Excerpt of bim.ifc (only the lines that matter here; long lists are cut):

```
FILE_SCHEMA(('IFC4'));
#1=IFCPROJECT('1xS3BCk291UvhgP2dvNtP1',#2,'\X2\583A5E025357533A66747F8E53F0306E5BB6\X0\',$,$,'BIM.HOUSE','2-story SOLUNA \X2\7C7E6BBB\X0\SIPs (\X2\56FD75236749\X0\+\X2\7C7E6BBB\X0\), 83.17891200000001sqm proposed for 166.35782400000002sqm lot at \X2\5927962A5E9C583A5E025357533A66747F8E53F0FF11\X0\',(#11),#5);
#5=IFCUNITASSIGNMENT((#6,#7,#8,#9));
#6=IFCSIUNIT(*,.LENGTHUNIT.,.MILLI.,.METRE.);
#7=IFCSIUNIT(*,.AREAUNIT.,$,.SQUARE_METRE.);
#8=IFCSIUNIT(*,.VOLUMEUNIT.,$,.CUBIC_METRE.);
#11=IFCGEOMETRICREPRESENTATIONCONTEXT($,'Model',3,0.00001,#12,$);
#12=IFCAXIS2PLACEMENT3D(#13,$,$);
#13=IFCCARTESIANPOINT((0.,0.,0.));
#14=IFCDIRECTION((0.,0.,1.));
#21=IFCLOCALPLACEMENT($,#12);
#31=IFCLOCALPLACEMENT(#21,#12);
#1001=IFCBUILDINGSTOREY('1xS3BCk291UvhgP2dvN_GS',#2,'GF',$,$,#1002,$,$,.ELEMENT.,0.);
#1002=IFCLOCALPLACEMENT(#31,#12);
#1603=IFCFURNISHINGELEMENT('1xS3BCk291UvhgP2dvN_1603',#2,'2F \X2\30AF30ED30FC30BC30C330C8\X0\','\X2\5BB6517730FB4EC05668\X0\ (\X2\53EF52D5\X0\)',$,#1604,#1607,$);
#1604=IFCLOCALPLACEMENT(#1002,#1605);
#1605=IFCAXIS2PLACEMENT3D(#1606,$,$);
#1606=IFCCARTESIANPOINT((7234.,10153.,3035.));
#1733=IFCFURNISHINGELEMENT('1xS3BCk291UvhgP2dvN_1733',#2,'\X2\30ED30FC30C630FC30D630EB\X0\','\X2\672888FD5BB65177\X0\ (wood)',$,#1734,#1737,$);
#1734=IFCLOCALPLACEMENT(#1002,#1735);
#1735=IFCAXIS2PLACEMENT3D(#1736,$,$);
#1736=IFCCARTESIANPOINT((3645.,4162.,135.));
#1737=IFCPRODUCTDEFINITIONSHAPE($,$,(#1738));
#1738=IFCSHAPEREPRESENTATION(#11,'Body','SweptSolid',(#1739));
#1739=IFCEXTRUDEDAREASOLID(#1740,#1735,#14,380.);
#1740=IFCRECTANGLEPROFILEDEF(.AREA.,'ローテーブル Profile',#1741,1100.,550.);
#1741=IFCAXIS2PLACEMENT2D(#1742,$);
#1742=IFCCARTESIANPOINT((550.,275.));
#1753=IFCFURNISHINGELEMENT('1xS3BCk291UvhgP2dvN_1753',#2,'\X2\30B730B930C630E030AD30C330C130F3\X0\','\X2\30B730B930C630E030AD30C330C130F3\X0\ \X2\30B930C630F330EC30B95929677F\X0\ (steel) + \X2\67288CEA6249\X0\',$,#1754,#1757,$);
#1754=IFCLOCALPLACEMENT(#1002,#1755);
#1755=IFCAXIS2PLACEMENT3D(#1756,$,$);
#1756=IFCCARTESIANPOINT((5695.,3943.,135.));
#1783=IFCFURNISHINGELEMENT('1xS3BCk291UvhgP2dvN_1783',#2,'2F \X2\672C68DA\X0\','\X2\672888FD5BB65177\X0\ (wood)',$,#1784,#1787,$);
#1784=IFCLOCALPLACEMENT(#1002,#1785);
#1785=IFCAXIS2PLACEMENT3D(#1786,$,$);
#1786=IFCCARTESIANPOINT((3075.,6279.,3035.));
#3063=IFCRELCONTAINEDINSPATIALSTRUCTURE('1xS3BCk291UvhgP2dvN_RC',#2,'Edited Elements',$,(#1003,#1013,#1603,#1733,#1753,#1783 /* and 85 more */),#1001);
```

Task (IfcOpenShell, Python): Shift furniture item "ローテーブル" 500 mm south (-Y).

```python
import ifcopenshell
import ifcopenshell.api.geometry
import ifcopenshell.util.placement
import ifcopenshell.util.unit

model = ifcopenshell.open("bim.ifc")
unit_scale = ifcopenshell.util.unit.calculate_unit_scale(model)

item = model.by_guid("1xS3BCk291UvhgP2dvN_1733")
matrix = ifcopenshell.util.placement.get_local_placement(item.ObjectPlacement)
matrix[1, 3] -= 0.5 / unit_scale
ifcopenshell.api.geometry.edit_object_placement(model, product=item, matrix=matrix, is_si=False)

print(ifcopenshell.util.placement.get_local_placement(item.ObjectPlacement).round(3) + 0.0)

model.write("bim_v2.ifc")
```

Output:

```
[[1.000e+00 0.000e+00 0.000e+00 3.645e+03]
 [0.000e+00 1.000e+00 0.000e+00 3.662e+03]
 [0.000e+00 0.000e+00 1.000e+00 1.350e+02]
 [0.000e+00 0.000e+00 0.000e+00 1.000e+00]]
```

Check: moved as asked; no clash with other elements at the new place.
